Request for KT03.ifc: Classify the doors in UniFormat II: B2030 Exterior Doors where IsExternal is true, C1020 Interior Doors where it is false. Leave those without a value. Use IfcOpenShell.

First a look at what the model holds.

```python
import ifcopenshell
import ifcopenshell.util.element

model = ifcopenshell.open("KT03.ifc")
print(model.schema)
print("classifications:", [c.Name for c in model.by_type("IfcClassification")])
values = [ifcopenshell.util.element.get_pset(e, "Pset_DoorCommon", "IsExternal") for e in model.by_type("IfcDoor")]
for value in (True, False, None):
    print("IsExternal", value, values.count(value))
```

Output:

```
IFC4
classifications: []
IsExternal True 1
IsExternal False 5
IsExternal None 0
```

```python
import ifcopenshell
import ifcopenshell.api.classification
import ifcopenshell.util.element

model = ifcopenshell.open("KT03.ifc")

system = ifcopenshell.api.classification.add_classification(model, classification="UniFormat II")

doors = model.by_type("IfcDoor")
external = {e: ifcopenshell.util.element.get_pset(e, "Pset_DoorCommon", "IsExternal") for e in doors}
for flag, code, name in ((True, "B2030", "Exterior Doors"), (False, "C1020", "Interior Doors")):
    products = [e for e in doors if external[e] is flag]
    ifcopenshell.api.classification.add_reference(
        model, products=products, classification=system, identification=code, name=name
    )
    print(code, len(products))

model.write("KT03_edited.ifc")
```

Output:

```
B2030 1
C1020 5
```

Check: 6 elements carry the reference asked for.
